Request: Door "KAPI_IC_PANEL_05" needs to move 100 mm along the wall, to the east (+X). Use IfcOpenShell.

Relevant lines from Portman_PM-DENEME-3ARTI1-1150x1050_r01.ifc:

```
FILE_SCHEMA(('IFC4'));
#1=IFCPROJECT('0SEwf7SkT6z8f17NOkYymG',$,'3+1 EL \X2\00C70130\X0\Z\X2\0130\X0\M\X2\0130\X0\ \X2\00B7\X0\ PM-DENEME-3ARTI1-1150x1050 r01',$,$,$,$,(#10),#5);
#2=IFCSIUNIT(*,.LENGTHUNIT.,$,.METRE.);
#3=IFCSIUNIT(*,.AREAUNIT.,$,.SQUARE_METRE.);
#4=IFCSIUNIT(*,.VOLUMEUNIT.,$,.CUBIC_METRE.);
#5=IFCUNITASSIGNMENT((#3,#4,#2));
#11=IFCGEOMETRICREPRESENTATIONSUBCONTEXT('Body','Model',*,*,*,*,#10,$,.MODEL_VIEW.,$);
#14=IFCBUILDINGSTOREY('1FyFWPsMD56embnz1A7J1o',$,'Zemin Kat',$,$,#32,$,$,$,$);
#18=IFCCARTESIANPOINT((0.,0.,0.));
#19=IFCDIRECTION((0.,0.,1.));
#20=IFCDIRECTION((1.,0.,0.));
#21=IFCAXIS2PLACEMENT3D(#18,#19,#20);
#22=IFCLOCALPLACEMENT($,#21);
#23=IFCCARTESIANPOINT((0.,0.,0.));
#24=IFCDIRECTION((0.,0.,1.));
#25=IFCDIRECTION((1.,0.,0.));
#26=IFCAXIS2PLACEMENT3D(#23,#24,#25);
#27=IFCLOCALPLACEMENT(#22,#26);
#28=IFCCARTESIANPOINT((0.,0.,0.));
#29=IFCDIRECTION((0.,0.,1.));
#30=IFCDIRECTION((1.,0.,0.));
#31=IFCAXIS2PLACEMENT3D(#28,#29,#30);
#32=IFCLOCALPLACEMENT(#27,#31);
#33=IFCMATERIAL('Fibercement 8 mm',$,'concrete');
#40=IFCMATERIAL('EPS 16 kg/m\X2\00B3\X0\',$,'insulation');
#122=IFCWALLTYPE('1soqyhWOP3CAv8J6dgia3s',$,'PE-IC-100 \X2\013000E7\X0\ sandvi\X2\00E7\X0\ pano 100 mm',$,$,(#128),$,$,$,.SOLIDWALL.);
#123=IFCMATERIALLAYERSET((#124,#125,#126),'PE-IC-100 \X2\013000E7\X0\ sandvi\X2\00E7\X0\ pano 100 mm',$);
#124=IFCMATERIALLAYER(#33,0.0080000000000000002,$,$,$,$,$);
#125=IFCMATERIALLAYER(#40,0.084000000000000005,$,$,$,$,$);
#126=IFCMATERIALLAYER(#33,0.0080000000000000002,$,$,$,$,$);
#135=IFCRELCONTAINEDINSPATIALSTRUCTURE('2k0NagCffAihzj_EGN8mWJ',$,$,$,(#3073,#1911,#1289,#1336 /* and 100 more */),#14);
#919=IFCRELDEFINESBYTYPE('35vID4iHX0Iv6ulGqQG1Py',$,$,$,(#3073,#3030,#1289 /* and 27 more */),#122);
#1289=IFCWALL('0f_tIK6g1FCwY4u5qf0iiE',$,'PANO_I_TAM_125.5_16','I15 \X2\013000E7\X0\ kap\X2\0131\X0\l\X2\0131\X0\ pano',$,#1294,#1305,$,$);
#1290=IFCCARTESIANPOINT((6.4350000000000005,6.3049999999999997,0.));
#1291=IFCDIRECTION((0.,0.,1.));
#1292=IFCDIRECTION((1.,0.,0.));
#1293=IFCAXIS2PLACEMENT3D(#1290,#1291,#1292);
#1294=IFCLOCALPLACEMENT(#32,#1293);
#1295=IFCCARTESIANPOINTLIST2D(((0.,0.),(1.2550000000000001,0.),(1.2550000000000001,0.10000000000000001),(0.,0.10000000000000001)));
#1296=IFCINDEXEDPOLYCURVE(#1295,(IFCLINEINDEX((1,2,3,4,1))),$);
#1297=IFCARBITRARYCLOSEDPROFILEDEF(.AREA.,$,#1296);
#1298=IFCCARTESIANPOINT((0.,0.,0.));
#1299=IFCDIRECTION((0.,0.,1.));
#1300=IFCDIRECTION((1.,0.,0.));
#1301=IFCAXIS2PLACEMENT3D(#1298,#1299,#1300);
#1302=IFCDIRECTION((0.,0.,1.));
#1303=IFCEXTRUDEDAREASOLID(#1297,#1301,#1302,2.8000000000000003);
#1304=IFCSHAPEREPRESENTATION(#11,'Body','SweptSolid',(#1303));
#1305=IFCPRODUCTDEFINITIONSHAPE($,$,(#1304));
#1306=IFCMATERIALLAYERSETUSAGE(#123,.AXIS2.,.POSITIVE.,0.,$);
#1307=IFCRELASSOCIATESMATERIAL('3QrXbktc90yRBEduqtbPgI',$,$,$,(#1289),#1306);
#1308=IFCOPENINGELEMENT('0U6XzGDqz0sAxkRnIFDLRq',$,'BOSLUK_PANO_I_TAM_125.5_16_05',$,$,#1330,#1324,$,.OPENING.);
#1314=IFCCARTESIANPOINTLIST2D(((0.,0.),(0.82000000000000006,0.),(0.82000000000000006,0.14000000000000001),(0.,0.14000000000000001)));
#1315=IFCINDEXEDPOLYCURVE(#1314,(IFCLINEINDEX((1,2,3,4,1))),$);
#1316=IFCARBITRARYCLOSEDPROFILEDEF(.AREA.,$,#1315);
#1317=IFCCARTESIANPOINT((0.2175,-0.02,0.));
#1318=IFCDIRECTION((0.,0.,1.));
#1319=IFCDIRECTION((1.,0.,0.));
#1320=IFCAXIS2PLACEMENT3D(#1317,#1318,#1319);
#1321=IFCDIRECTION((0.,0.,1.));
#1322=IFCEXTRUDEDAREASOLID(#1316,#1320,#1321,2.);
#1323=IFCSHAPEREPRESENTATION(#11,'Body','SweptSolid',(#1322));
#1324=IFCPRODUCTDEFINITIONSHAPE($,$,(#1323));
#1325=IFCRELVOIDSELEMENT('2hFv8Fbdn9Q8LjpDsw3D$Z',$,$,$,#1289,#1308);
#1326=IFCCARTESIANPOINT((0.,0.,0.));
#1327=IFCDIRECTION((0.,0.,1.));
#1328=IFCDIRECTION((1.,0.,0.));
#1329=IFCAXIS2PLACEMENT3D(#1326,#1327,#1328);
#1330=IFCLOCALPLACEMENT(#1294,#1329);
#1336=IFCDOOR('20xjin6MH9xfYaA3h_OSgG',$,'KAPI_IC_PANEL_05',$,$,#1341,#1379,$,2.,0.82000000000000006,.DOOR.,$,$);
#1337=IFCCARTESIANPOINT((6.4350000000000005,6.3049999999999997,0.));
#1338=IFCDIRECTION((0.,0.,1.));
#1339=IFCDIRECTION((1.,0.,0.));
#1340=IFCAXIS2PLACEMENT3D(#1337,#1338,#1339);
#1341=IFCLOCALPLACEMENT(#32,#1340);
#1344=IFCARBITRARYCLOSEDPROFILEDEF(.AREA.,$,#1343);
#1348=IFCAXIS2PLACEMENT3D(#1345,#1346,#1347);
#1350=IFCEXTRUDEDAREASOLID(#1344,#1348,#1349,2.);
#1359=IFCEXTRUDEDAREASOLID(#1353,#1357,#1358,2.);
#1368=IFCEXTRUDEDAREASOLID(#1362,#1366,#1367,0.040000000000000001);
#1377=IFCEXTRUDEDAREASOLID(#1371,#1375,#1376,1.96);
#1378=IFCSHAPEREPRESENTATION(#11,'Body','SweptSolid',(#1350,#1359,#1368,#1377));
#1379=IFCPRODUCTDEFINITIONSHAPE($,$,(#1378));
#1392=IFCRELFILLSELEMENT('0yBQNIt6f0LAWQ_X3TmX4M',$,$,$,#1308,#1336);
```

```python
import ifcopenshell
import ifcopenshell.api.geometry
import ifcopenshell.util.placement

model = ifcopenshell.open("Portman_PM-DENEME-3ARTI1-1150x1050_r01.ifc")

door = model.by_guid("20xjin6MH9xfYaA3h_OSgG")
opening = door.FillsVoids[0].RelatingOpeningElement
wall = opening.VoidsElements[0].RelatingBuildingElement

wall_matrix = ifcopenshell.util.placement.get_local_placement(wall.ObjectPlacement)
shift = wall_matrix[:3, 0] * 0.1
before = ifcopenshell.util.placement.get_local_placement(door.ObjectPlacement)[:3, 3].copy()

# The door is not placed relative to its opening, so move both.
for product in (opening, door):
    matrix = ifcopenshell.util.placement.get_local_placement(product.ObjectPlacement)
    matrix[:3, 3] += shift
    ifcopenshell.api.geometry.edit_object_placement(model, product=product, matrix=matrix, is_si=False)

after = ifcopenshell.util.placement.get_local_placement(door.ObjectPlacement)[:3, 3]
print("door moved by", (after - before).round(3) + 0.0)

model.write("Portman_PM-DENEME-3ARTI1-1150x1050_r01_v2.ifc")
```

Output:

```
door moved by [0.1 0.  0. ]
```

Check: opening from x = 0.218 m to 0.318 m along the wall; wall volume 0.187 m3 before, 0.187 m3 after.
